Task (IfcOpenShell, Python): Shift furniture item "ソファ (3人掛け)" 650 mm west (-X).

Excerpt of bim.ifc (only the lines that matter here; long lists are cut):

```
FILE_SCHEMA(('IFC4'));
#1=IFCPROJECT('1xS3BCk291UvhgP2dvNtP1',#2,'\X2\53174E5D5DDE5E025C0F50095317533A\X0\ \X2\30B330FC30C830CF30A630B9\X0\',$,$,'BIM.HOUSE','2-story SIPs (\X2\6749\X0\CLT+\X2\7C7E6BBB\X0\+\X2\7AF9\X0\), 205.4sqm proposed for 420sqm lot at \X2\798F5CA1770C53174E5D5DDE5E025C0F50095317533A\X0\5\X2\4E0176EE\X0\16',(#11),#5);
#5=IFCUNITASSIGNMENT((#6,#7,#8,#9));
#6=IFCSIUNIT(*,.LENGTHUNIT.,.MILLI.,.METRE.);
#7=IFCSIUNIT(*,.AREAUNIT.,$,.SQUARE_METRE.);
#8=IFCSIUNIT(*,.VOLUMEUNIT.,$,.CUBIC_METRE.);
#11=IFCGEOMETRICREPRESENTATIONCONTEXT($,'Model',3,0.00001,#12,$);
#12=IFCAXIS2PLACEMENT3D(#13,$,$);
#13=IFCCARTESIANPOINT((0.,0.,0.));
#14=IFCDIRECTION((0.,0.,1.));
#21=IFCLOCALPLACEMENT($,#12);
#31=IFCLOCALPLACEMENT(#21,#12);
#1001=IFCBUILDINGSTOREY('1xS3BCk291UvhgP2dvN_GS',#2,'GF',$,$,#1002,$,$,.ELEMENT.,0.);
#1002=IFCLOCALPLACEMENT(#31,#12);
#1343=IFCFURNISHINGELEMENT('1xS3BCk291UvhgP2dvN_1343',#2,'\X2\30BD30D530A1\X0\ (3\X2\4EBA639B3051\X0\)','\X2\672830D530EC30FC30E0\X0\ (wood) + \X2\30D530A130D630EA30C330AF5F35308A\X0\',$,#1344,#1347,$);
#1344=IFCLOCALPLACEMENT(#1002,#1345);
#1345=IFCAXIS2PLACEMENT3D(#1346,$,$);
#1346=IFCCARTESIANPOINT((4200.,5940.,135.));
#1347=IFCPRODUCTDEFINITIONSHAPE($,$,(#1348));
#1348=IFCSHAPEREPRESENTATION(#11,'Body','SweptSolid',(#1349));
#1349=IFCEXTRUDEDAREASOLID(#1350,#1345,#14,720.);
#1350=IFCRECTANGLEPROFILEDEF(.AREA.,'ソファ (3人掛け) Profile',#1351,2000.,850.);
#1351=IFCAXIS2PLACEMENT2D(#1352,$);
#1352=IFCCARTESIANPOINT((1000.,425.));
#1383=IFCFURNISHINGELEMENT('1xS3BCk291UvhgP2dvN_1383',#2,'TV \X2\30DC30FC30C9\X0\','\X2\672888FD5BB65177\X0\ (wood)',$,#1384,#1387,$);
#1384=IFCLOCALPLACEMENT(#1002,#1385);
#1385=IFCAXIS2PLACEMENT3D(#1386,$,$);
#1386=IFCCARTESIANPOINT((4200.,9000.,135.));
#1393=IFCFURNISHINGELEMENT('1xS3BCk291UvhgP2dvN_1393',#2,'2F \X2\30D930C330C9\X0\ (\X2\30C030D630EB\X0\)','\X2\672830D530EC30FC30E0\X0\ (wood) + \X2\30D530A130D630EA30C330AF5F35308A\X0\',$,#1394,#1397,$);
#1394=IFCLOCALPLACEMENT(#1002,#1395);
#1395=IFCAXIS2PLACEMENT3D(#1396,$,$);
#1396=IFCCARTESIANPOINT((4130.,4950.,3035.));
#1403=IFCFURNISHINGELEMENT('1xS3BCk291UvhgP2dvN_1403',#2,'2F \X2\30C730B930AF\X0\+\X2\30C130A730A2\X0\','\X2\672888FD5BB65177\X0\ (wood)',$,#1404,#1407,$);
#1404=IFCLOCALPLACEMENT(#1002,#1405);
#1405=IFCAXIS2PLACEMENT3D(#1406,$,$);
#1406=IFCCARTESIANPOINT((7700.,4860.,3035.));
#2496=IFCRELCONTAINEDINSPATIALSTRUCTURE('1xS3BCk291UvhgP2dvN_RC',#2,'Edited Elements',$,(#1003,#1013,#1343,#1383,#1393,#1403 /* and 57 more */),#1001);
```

```python
import ifcopenshell
import ifcopenshell.api.geometry
import ifcopenshell.util.placement
import ifcopenshell.util.unit

model = ifcopenshell.open("bim.ifc")
unit_scale = ifcopenshell.util.unit.calculate_unit_scale(model)

item = model.by_guid("1xS3BCk291UvhgP2dvN_1343")
matrix = ifcopenshell.util.placement.get_local_placement(item.ObjectPlacement)
matrix[0, 3] -= 0.65 / unit_scale
ifcopenshell.api.geometry.edit_object_placement(model, product=item, matrix=matrix, is_si=False)

print(ifcopenshell.util.placement.get_local_placement(item.ObjectPlacement).round(3) + 0.0)

model.write("bim-out.ifc")
```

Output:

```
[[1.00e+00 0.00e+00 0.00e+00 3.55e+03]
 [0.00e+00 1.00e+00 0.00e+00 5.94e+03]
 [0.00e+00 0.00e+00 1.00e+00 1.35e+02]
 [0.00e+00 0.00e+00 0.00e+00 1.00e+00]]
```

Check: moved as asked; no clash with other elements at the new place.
